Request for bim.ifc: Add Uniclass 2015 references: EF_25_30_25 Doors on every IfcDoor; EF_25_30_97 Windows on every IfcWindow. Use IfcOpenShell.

First a look at what the model holds.

```python
import ifcopenshell

model = ifcopenshell.open("bim.ifc")
print(model.schema)
print("classifications:", [c.Name for c in model.by_type("IfcClassification")])
for ifc_class in ("IfcDoor", "IfcRoof", "IfcStair", "IfcWall", "IfcWindow"):
    print(ifc_class, len(model.by_type(ifc_class)))
```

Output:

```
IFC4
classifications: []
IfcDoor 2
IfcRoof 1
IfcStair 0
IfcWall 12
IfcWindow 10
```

```python
import ifcopenshell
import ifcopenshell.api.classification

model = ifcopenshell.open("bim.ifc")

system = ifcopenshell.api.classification.add_classification(model, classification="Uniclass 2015")

codes = {
    "IfcDoor": ("EF_25_30_25", "Doors"),
    "IfcWindow": ("EF_25_30_97", "Windows"),
}
for ifc_class, (code, name) in codes.items():
    products = model.by_type(ifc_class)
    ifcopenshell.api.classification.add_reference(
        model, products=products, classification=system, identification=code, name=name
    )
    print(code, len(products))

model.write("bim_edited.ifc")
```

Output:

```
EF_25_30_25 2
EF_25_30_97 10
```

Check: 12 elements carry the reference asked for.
